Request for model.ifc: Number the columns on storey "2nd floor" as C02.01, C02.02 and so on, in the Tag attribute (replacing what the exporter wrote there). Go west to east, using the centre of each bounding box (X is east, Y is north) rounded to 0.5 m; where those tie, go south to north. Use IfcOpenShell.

First a look at what the model holds.

```python
import ifcopenshell
import ifcopenshell.util.element
import ifcopenshell.util.placement

model = ifcopenshell.open("model.ifc")
print(model.schema)
storey = next(s for s in model.by_type("IfcBuildingStorey") if s.Name == "2nd floor")
columns = [e for e in ifcopenshell.util.element.get_decomposition(storey) if e.is_a("IfcColumn")]
for e in sorted(columns, key=lambda e: e.id()):
    origin = ifcopenshell.util.placement.get_local_placement(e.ObjectPlacement)[:3, 3]
    print(e.id(), e.Tag, e.Name, origin.round(2) + 0.0, sep=" | ")
```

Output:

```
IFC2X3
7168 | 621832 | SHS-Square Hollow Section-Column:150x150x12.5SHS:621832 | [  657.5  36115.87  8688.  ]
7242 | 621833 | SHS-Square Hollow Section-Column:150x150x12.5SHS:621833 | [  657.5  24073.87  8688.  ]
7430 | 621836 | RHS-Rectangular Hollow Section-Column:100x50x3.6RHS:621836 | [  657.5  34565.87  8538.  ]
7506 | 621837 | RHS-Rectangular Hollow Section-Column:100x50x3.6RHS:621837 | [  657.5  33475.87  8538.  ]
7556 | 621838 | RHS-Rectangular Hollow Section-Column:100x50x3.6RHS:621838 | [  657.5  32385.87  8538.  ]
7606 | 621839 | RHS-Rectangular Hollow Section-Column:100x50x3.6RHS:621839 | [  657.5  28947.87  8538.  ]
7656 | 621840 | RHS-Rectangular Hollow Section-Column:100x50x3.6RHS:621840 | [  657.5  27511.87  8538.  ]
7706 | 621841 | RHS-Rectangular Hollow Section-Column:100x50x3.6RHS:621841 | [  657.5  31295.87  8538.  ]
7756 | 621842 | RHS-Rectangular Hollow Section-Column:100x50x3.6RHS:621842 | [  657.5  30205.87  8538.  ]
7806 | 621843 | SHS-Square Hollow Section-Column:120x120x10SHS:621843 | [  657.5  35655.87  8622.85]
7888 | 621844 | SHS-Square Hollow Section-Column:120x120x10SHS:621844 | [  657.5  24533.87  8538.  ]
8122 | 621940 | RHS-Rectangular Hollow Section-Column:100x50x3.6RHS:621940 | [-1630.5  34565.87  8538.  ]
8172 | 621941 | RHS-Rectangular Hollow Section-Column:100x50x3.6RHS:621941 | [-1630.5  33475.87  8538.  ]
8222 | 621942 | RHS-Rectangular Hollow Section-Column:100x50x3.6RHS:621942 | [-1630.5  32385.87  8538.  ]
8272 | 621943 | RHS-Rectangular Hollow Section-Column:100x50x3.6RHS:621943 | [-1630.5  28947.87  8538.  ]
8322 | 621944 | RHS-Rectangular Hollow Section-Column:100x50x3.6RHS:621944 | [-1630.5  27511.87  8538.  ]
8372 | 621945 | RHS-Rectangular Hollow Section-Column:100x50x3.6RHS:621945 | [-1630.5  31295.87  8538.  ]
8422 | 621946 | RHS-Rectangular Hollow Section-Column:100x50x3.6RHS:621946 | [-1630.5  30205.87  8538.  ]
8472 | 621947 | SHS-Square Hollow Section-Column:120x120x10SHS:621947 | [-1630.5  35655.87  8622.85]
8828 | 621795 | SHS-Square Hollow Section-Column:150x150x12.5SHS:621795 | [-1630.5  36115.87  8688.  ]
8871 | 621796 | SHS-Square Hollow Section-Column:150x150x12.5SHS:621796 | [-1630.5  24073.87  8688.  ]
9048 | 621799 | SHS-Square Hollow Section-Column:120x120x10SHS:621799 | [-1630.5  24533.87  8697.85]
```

```python
import ifcopenshell
import ifcopenshell.geom
import ifcopenshell.util.element
import ifcopenshell.util.shape

model = ifcopenshell.open("model.ifc")
settings = ifcopenshell.geom.settings()
settings.set("use-world-coords", True)


def centre(element):
    shape = ifcopenshell.geom.create_shape(settings, element)
    return ifcopenshell.util.shape.get_bbox_centroid(shape.geometry)


storey = next(s for s in model.by_type("IfcBuildingStorey") if s.Name == "2nd floor")
columns = [e for e in ifcopenshell.util.element.get_decomposition(storey) if e.is_a("IfcColumn")]

# Insertion points can sit at a corner or the storey origin, so sort by the geometry (in metres).
centres = {e: centre(e) for e in columns}
columns.sort(key=lambda e: (round(centres[e][0] / 0.5), centres[e][1]))

for i, e in enumerate(columns, start=1):
    number = f"C02.{i:02d}"
    e.Tag = number
    print(e.id(), number)

model.write("model-out.ifc")
```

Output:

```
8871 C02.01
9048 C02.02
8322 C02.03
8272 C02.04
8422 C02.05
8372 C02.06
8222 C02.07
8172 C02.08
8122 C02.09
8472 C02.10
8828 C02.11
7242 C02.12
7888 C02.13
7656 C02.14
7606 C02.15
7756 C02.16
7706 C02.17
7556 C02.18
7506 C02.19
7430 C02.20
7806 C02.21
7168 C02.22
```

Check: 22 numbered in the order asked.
